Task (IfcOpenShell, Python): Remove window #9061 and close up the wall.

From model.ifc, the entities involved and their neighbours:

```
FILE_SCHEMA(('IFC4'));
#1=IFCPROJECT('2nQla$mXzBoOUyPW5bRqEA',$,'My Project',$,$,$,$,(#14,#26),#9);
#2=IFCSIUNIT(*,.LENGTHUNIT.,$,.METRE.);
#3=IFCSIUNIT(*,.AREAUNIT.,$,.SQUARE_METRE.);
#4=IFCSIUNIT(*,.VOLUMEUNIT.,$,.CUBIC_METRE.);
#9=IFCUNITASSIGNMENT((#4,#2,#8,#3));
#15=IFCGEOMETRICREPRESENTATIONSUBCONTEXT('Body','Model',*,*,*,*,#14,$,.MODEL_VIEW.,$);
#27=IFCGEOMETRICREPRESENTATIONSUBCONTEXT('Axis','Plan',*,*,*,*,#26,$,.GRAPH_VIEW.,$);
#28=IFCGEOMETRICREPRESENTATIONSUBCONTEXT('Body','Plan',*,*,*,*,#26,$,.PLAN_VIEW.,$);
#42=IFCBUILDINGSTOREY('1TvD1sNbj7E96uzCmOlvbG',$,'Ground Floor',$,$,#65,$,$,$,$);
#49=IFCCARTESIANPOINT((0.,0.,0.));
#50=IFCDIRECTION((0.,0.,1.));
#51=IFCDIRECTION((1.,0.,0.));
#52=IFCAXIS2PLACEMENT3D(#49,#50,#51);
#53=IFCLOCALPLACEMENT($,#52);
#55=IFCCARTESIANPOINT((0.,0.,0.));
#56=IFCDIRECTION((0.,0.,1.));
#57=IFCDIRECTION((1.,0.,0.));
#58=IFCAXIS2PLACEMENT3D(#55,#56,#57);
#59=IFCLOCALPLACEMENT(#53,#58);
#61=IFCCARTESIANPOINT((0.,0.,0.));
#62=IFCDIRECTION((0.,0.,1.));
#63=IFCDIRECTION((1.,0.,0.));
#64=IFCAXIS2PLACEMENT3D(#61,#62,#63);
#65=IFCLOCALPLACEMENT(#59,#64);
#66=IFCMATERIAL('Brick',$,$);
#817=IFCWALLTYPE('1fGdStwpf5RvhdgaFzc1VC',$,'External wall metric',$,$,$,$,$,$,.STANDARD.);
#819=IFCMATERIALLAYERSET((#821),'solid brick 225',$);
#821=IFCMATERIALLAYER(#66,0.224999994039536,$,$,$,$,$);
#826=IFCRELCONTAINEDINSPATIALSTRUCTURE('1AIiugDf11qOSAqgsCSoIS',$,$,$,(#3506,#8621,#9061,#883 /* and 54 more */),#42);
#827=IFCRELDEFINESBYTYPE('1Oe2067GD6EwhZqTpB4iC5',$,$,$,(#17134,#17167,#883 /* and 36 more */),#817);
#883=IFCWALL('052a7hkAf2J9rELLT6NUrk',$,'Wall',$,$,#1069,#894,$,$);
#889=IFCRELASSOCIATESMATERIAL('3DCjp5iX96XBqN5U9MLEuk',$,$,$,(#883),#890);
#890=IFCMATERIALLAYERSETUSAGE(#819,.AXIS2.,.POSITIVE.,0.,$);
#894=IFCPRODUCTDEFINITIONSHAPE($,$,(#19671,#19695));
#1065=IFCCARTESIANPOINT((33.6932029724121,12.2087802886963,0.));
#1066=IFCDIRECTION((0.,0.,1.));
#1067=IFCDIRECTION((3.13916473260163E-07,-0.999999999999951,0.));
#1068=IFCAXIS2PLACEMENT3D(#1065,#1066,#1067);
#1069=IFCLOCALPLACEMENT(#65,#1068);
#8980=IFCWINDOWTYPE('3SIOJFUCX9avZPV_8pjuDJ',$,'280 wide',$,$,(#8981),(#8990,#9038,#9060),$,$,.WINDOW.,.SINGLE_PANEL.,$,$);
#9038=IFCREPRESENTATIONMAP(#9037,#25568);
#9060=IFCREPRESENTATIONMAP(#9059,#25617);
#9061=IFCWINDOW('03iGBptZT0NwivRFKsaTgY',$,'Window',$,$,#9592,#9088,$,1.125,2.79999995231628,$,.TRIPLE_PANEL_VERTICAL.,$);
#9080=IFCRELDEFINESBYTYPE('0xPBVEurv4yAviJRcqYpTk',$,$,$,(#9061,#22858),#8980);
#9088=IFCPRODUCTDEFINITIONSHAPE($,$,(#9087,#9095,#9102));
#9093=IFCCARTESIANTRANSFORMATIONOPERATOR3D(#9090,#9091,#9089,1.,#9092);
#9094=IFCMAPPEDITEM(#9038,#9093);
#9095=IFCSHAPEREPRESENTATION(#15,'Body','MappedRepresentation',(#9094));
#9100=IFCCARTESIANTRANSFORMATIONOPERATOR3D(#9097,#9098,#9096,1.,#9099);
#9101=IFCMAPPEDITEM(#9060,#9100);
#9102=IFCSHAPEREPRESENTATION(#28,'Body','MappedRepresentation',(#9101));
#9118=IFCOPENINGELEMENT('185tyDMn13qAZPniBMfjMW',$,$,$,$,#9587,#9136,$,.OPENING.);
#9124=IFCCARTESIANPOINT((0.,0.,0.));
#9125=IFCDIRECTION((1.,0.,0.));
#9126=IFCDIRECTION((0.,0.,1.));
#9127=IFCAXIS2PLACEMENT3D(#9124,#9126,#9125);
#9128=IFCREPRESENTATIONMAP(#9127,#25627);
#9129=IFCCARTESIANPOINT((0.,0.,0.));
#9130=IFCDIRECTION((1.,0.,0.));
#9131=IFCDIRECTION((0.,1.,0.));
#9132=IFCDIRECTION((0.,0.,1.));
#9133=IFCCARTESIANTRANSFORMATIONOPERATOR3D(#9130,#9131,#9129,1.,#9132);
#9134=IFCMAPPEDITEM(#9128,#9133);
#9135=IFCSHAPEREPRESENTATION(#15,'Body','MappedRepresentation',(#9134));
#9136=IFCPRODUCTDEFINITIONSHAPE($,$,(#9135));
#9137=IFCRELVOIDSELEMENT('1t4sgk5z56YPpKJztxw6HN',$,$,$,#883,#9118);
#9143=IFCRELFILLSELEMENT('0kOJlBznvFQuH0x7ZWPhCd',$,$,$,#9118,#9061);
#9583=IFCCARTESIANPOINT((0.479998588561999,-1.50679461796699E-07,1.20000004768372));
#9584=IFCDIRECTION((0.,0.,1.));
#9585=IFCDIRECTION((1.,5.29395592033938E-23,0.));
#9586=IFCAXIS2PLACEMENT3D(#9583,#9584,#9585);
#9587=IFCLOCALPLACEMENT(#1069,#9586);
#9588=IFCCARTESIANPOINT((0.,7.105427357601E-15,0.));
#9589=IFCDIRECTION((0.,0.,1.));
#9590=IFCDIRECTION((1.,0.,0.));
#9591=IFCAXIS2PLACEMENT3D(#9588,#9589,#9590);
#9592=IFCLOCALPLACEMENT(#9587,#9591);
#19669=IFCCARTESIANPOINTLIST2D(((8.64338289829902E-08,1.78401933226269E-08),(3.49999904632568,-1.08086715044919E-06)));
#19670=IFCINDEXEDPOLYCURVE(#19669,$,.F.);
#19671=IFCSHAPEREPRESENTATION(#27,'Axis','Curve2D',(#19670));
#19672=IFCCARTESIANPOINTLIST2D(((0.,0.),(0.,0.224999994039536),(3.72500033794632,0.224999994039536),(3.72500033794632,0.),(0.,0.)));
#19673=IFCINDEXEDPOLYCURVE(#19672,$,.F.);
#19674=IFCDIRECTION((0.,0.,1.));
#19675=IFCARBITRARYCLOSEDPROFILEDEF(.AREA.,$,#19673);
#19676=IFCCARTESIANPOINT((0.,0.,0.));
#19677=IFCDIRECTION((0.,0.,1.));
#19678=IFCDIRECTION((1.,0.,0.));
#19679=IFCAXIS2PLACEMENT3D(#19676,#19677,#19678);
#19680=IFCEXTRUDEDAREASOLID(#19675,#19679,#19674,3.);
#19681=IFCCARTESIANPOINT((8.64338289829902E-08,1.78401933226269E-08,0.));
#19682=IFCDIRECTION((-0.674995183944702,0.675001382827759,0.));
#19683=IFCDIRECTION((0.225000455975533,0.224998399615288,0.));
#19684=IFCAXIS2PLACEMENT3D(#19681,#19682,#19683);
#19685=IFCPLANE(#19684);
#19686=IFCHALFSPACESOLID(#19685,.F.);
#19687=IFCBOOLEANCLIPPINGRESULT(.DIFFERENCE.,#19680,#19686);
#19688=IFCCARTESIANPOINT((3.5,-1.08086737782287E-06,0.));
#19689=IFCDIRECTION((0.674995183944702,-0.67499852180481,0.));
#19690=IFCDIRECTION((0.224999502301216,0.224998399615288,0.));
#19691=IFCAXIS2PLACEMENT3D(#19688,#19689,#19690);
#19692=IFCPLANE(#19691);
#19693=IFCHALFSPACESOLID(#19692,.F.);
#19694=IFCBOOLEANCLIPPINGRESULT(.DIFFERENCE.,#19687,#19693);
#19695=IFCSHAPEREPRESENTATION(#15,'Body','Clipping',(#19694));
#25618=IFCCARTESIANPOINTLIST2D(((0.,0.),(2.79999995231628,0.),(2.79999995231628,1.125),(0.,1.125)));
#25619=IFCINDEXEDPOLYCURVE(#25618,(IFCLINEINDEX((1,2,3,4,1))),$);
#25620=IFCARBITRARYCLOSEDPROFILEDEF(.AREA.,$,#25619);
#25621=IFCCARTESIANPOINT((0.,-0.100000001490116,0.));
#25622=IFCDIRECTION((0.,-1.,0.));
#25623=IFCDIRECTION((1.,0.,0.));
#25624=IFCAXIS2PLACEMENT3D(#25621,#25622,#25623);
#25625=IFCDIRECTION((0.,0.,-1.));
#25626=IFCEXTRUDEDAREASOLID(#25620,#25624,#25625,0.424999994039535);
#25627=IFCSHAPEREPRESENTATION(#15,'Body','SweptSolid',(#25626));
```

```python
import ifcopenshell
import ifcopenshell.api.feature
import ifcopenshell.api.root
import ifcopenshell.geom
import ifcopenshell.util.shape

model = ifcopenshell.open("model.ifc")
settings = ifcopenshell.geom.settings()


def volume(element):
    """Net volume in cubic metres, openings subtracted."""
    shape = ifcopenshell.geom.create_shape(settings, element)
    return ifcopenshell.util.shape.get_volume(shape.geometry)


window = model.by_id(9061)
opening = window.FillsVoids[0].RelatingOpeningElement
wall = opening.VoidsElements[0].RelatingBuildingElement
before = volume(wall)

ifcopenshell.api.root.remove_product(model, product=window)
ifcopenshell.api.feature.remove_feature(model, feature=opening)

after = volume(wall)

print(f"wall volume {before:.3f} -> {after:.3f} m3")

model.write("model_edited.ifc")
```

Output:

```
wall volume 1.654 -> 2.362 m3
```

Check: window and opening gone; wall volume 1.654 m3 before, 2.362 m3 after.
